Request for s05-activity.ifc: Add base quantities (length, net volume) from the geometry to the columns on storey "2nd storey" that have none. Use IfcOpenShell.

First a look at what the model holds.

```python
import ifcopenshell
import ifcopenshell.util.element
import ifcopenshell.util.unit

model = ifcopenshell.open("s05-activity.ifc")
print(model.schema)
for unit_type in ("LENGTHUNIT", "AREAUNIT", "VOLUMEUNIT"):
    print(unit_type, ifcopenshell.util.unit.calculate_unit_scale(model, unit_type))
storey = next(s for s in model.by_type("IfcBuildingStorey") if s.Name == "2nd storey")
columns = [e for e in ifcopenshell.util.element.get_decomposition(storey) if e.is_a("IfcColumn")]
for e in sorted(columns, key=lambda e: e.id()):
    print(e.id(), e.is_a(), e.Name, list(ifcopenshell.util.element.get_psets(e, qtos_only=True)), sep=" | ")
```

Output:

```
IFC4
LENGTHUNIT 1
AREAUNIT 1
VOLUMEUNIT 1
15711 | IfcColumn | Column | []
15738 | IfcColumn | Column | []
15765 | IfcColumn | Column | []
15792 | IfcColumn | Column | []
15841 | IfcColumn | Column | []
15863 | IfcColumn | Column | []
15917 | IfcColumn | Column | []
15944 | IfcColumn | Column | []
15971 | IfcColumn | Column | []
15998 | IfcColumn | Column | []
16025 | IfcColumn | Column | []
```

```python
import ifcopenshell
import ifcopenshell.api.pset
import ifcopenshell.geom
import ifcopenshell.util.element
import ifcopenshell.util.shape
import ifcopenshell.util.unit

model = ifcopenshell.open("s05-activity.ifc")
unit_scale = ifcopenshell.util.unit.calculate_unit_scale(model)
volume_scale = ifcopenshell.util.unit.calculate_unit_scale(model, "VOLUMEUNIT")
settings = ifcopenshell.geom.settings()

storey = next(s for s in model.by_type("IfcBuildingStorey") if s.Name == "2nd storey")
columns = [e for e in ifcopenshell.util.element.get_decomposition(storey) if e.is_a("IfcColumn")]

for e in sorted(columns, key=lambda e: e.id()):
    if ifcopenshell.util.element.get_psets(e, qtos_only=True, should_inherit=False):
        continue
    # Geometry comes back in metres, in the element's own axes.
    shape = ifcopenshell.geom.create_shape(settings, e)
    values = {
        "Length": ifcopenshell.util.shape.get_z(shape.geometry) / unit_scale,
        "NetVolume": ifcopenshell.util.shape.get_volume(shape.geometry) / volume_scale,
    }
    qto = ifcopenshell.api.pset.add_qto(model, product=e, name="Qto_ColumnBaseQuantities")
    ifcopenshell.api.pset.edit_qto(model, qto=qto, properties=values)
    print(e.id(), {k: round(v, 3) for k, v in values.items()})

model.write("s05-activity_updated.ifc")
```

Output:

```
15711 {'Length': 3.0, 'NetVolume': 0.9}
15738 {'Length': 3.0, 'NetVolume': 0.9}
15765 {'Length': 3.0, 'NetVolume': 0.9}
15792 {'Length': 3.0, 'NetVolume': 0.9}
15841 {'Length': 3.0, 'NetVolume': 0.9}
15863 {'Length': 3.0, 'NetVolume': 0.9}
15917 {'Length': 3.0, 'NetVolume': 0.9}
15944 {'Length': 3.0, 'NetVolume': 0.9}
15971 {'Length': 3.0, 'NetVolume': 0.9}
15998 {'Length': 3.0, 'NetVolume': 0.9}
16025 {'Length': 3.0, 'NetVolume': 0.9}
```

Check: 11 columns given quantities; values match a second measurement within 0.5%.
